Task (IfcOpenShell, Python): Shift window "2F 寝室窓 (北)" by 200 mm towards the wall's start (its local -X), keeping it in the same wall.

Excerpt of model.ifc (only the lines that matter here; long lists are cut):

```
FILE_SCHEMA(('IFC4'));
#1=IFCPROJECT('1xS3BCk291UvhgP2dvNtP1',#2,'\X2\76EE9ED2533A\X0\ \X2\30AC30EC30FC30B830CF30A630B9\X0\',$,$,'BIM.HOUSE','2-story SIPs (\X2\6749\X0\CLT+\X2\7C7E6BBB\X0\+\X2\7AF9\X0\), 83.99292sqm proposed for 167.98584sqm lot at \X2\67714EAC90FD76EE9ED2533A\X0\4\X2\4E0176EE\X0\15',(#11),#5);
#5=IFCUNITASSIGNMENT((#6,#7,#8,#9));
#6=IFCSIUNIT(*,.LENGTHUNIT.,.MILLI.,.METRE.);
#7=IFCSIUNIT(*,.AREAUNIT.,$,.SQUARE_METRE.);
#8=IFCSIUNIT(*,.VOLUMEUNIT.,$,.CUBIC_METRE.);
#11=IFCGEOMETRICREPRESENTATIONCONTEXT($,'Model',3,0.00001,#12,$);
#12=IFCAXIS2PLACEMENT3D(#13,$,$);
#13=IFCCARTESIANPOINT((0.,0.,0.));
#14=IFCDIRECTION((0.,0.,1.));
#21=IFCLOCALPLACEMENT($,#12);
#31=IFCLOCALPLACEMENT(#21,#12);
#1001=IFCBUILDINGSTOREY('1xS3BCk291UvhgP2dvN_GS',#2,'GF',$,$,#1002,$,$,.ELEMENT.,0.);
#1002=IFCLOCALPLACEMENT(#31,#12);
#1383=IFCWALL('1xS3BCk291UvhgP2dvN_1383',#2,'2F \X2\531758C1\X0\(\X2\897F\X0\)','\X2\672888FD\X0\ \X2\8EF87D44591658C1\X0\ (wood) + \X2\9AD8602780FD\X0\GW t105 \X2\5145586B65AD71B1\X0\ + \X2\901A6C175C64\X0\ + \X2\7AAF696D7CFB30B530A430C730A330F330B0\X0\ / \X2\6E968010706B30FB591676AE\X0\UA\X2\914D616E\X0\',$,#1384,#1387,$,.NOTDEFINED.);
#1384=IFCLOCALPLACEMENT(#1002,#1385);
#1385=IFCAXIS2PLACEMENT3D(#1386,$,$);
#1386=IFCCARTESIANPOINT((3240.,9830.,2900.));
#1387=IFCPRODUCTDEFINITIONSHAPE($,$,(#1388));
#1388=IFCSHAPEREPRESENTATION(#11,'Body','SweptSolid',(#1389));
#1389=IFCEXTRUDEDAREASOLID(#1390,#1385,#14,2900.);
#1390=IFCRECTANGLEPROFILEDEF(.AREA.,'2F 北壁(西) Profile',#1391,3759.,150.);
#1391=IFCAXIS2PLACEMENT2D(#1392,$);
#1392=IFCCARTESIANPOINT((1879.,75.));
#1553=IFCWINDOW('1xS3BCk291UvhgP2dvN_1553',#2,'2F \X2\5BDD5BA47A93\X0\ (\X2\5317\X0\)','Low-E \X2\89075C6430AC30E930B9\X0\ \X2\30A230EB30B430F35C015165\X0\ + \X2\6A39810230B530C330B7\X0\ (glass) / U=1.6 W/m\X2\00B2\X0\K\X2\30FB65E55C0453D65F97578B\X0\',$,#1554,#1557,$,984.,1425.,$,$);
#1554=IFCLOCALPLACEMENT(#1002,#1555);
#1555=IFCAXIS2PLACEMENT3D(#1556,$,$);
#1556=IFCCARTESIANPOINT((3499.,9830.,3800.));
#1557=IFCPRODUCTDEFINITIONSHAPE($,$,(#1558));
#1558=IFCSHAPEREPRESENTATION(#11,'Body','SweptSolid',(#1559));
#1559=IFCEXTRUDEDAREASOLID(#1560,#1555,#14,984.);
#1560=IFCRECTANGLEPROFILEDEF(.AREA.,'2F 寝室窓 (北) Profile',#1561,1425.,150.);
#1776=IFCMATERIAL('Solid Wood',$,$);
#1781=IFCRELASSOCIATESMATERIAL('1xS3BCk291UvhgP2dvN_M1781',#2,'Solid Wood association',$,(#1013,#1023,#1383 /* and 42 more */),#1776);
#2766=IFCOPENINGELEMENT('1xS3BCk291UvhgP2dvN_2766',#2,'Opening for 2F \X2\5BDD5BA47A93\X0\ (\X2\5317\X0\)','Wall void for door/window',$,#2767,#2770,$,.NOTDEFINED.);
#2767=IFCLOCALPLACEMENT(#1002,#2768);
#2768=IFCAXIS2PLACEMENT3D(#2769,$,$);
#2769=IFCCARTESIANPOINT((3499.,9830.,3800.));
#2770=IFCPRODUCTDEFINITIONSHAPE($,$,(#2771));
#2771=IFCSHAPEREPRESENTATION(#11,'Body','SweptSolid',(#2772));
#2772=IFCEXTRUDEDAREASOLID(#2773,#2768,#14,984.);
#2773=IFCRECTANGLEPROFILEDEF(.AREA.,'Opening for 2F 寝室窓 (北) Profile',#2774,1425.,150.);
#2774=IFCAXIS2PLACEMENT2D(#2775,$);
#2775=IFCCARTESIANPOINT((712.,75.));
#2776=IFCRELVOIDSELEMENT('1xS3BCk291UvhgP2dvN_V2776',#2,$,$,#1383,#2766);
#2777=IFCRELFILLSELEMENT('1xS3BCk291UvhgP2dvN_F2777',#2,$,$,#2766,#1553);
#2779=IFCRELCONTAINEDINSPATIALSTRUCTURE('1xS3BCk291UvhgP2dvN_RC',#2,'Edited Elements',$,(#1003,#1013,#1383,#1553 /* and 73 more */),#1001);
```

```python
import ifcopenshell
import ifcopenshell.api.geometry
import ifcopenshell.util.placement

model = ifcopenshell.open("model.ifc")

window = model.by_guid("1xS3BCk291UvhgP2dvN_1553")
opening = window.FillsVoids[0].RelatingOpeningElement
wall = opening.VoidsElements[0].RelatingBuildingElement

wall_matrix = ifcopenshell.util.placement.get_local_placement(wall.ObjectPlacement)
shift = wall_matrix[:3, 0] * -200.0
before = ifcopenshell.util.placement.get_local_placement(window.ObjectPlacement)[:3, 3].copy()

# The window is not placed relative to its opening, so move both.
for product in (opening, window):
    matrix = ifcopenshell.util.placement.get_local_placement(product.ObjectPlacement)
    matrix[:3, 3] += shift
    ifcopenshell.api.geometry.edit_object_placement(model, product=product, matrix=matrix, is_si=False)

after = ifcopenshell.util.placement.get_local_placement(window.ObjectPlacement)[:3, 3]
print("window moved by", (after - before).round(3) + 0.0)

model.write("model_rev.ifc")
```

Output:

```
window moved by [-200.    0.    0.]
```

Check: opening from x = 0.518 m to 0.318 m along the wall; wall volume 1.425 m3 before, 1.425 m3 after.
